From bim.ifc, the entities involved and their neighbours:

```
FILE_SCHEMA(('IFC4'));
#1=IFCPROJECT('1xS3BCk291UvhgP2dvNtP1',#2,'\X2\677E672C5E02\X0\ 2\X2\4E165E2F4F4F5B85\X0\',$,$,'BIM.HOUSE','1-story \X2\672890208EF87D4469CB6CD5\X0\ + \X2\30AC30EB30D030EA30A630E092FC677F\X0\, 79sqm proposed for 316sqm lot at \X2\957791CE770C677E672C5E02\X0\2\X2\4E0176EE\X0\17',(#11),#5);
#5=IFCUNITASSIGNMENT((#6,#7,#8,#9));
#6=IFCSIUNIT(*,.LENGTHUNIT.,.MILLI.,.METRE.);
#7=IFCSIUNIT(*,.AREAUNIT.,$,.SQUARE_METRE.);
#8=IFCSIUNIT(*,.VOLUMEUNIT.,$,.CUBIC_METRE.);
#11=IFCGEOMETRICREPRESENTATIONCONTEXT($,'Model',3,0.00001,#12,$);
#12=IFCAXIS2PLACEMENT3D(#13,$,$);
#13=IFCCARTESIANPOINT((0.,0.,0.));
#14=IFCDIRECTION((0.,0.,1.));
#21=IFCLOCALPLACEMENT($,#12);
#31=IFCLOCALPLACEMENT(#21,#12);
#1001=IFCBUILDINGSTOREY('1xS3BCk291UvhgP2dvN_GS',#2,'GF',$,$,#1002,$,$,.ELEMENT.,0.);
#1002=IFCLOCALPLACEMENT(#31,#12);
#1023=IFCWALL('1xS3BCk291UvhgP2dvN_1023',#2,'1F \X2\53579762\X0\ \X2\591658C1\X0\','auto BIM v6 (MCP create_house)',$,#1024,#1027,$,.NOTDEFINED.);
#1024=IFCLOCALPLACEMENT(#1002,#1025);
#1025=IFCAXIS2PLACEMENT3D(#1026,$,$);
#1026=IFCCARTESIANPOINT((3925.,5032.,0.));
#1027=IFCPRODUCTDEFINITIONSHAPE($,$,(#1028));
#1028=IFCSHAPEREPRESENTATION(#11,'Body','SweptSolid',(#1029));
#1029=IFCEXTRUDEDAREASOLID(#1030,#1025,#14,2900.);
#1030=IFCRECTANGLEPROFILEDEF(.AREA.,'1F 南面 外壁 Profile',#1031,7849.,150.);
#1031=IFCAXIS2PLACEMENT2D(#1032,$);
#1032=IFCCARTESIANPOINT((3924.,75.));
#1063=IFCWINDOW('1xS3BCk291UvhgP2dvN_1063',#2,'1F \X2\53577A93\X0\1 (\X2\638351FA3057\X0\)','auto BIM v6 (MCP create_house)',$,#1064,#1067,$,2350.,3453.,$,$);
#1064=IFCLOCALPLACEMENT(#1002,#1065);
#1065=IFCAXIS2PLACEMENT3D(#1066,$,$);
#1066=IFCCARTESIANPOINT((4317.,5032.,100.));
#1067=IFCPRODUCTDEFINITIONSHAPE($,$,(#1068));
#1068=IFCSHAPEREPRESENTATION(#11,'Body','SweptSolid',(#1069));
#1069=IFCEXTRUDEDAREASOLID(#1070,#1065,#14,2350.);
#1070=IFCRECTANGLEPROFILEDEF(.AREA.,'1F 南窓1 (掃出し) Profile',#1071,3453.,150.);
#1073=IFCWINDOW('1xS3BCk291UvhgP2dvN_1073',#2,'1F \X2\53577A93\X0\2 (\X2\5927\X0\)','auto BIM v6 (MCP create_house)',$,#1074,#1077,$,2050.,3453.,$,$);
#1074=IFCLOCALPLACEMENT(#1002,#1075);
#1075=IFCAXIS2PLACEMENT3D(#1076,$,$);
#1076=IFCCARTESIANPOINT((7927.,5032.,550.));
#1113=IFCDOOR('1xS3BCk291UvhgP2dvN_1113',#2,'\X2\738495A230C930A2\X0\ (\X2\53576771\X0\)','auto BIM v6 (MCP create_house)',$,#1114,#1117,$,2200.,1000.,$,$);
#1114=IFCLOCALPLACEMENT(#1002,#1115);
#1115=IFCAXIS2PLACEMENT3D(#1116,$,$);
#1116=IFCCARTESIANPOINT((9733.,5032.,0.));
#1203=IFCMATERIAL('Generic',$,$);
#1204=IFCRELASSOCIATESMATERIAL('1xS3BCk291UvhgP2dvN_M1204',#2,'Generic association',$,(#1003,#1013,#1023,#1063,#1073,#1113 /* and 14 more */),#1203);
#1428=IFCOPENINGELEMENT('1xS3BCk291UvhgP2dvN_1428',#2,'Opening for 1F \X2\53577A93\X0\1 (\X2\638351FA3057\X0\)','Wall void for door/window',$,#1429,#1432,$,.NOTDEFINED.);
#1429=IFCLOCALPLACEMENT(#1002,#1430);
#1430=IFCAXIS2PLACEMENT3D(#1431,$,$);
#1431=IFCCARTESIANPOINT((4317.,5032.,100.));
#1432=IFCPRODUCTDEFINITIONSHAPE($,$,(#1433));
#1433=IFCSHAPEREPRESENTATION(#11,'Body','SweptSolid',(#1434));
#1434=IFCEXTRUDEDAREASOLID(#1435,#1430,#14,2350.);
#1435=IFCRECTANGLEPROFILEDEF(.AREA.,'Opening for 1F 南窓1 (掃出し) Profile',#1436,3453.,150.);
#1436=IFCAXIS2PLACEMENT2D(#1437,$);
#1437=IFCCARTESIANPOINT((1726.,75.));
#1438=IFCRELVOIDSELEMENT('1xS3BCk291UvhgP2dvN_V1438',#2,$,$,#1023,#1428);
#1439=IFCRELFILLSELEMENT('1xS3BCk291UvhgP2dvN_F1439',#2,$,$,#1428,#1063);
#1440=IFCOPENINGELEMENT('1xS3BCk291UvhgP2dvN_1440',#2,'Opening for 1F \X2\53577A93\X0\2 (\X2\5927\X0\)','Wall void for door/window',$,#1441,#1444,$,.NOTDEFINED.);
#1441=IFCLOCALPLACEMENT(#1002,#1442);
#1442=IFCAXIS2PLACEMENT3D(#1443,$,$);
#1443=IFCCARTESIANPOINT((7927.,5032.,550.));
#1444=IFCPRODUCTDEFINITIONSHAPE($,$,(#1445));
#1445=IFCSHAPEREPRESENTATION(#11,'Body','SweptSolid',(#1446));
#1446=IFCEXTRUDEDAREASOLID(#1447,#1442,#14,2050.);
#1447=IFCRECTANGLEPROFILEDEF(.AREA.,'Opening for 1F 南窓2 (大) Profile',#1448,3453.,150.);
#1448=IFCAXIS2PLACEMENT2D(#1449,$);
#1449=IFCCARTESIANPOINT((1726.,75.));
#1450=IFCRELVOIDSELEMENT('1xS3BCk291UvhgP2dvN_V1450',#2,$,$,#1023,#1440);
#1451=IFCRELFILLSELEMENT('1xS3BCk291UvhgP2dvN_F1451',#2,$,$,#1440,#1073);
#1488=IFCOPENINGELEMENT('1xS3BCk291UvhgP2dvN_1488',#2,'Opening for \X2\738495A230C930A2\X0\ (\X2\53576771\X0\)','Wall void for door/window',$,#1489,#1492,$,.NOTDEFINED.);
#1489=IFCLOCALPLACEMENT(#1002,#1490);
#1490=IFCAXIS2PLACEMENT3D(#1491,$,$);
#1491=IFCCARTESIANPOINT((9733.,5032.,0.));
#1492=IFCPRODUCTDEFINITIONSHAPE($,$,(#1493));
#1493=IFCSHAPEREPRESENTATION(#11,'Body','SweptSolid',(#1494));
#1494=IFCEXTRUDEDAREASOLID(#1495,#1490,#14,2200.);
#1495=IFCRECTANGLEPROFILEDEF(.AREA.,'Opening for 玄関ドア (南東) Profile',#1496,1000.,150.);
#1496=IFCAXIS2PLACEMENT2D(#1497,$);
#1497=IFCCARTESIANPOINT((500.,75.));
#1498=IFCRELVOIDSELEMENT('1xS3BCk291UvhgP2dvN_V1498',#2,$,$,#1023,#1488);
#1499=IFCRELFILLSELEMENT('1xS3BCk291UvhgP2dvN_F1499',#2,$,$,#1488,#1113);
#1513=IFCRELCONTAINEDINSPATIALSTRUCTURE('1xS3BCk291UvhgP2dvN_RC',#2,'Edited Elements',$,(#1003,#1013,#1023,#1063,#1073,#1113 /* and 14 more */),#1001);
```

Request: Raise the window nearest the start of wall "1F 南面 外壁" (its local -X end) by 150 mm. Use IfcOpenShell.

```python
import numpy as np
import ifcopenshell
import ifcopenshell.api.geometry
import ifcopenshell.util.placement
import ifcopenshell.util.unit

model = ifcopenshell.open("bim.ifc")
unit_scale = ifcopenshell.util.unit.calculate_unit_scale(model)

window = model.by_id(1063)
opening = window.FillsVoids[0].RelatingOpeningElement
dz = 0.15 / unit_scale

shift = np.array([0.0, 0.0, dz])
# The window is not placed relative to its opening, so move both.
for product in (opening, window):
    matrix = ifcopenshell.util.placement.get_local_placement(product.ObjectPlacement)
    matrix[:3, 3] += shift
    ifcopenshell.api.geometry.edit_object_placement(model, product=product, matrix=matrix, is_si=False)

print(f"moved by {dz * unit_scale:+.3f} m")

model.write("bim-out.ifc")
```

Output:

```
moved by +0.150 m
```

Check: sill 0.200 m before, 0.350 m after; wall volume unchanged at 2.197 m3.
